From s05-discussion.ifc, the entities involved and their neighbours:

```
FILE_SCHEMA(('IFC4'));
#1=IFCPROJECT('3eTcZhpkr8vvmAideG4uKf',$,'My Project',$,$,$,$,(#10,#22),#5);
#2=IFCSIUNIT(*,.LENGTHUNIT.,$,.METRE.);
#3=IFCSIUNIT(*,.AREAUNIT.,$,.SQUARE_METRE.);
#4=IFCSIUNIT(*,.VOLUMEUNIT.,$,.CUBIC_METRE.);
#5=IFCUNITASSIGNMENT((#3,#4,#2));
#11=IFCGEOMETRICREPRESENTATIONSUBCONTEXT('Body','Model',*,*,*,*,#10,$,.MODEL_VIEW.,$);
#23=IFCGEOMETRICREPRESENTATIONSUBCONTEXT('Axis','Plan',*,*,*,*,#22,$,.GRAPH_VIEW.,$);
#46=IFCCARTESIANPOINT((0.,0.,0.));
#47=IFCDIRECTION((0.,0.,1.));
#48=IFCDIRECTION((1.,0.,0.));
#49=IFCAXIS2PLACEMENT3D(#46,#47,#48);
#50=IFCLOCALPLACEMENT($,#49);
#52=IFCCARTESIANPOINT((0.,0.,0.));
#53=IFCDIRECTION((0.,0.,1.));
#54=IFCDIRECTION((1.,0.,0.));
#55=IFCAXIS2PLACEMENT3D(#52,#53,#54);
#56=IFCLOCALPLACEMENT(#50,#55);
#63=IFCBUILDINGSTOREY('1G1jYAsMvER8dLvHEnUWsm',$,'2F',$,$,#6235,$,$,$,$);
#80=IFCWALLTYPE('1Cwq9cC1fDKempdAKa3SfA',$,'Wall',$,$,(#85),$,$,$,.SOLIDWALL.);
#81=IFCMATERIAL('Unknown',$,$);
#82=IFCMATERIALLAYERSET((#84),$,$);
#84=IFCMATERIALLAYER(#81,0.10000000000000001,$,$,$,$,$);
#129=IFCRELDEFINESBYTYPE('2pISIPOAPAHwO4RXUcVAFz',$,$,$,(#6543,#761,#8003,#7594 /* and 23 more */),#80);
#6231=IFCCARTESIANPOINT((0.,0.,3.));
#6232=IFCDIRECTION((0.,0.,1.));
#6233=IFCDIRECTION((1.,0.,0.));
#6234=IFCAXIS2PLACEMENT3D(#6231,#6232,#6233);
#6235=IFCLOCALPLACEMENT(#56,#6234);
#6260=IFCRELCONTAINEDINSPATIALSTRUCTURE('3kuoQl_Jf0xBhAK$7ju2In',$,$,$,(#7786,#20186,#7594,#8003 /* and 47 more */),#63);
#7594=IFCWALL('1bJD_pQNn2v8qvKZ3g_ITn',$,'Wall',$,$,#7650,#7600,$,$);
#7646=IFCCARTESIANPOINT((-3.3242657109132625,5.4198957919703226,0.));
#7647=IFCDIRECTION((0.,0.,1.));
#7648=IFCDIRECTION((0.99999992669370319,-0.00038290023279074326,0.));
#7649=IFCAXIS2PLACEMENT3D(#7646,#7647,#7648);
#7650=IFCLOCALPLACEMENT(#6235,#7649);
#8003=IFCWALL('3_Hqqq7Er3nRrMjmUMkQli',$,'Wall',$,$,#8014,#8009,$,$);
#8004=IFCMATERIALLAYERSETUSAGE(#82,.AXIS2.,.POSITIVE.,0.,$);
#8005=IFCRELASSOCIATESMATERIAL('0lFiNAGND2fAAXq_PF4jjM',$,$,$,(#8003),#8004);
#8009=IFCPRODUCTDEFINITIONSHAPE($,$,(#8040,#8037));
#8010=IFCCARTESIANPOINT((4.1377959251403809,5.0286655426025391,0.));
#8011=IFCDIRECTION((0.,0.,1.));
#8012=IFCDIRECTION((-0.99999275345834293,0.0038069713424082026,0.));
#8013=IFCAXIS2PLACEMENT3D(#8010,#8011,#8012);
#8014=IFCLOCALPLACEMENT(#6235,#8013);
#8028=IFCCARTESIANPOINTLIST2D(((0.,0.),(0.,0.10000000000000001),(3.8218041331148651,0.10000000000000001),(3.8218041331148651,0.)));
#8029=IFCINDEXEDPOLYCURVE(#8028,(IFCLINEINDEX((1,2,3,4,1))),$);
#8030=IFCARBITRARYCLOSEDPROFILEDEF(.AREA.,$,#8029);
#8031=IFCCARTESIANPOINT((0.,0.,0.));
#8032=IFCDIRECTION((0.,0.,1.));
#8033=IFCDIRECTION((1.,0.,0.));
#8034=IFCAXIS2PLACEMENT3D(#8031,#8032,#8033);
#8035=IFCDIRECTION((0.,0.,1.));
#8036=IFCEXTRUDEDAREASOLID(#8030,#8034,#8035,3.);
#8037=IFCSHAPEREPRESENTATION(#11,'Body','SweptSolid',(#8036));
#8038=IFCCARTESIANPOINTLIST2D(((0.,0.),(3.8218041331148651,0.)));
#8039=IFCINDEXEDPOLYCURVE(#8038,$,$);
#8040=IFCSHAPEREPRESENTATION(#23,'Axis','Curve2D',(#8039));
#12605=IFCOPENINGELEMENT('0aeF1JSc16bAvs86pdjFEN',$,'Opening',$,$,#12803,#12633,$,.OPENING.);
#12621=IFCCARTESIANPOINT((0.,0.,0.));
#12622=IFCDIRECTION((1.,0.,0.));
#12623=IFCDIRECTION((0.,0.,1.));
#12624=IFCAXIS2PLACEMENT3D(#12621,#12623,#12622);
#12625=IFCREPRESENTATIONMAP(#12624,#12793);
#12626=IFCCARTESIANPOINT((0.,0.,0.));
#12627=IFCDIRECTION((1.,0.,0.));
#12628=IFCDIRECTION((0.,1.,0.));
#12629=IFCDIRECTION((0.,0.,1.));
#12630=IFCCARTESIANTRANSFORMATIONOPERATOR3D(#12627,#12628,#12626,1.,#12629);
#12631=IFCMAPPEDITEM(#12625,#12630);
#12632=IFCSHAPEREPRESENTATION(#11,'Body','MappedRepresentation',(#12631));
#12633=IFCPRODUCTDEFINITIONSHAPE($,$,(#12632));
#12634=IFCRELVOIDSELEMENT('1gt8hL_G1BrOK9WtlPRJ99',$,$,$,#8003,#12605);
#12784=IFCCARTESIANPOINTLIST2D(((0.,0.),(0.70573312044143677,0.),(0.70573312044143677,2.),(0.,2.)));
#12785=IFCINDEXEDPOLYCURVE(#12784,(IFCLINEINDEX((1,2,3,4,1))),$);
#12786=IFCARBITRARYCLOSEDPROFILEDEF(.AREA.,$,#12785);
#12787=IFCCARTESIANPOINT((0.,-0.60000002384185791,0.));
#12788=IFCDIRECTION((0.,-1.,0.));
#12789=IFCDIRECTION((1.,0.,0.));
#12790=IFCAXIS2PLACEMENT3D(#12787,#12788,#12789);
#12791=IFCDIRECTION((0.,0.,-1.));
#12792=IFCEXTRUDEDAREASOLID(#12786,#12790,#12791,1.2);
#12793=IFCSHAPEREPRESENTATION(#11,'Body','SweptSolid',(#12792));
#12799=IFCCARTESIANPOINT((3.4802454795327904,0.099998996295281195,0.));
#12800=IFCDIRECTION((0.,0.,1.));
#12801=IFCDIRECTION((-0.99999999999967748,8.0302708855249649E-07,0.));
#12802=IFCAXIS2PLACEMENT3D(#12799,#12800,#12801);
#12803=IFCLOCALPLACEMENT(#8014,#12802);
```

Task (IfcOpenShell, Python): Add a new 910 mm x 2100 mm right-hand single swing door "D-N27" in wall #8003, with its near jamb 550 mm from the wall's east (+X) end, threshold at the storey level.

```python
import numpy as np
import ifcopenshell
import ifcopenshell.api.feature
import ifcopenshell.api.geometry
import ifcopenshell.api.root
import ifcopenshell.api.spatial
import ifcopenshell.geom
import ifcopenshell.util.element
import ifcopenshell.util.placement
import ifcopenshell.util.representation
import ifcopenshell.util.shape
import ifcopenshell.util.unit

model = ifcopenshell.open("s05-discussion.ifc")
unit_scale = ifcopenshell.util.unit.calculate_unit_scale(model)
settings = ifcopenshell.geom.settings()


def volume(element):
    """Net volume in cubic metres, openings subtracted."""
    shape = ifcopenshell.geom.create_shape(settings, element)
    return ifcopenshell.util.shape.get_volume(shape.geometry)


wall = model.by_id(8003)
storey = ifcopenshell.util.element.get_container(wall, ifc_class="IfcBuildingStorey")
context = ifcopenshell.util.representation.get_context(model, "Model", "Body", "MODEL_VIEW")
before = volume(wall)

width, height, from_end, sill = 0.91, 2.1, 0.55, 0.0  # metres

# The wall runs along its own X axis, and the end named is its -X end.
wall_shape = ifcopenshell.geom.create_shape(settings, wall)
x, y, z = ifcopenshell.util.shape.get_vertices(wall_shape.geometry).T
start = x.min() + from_end
face, thickness = float(y.min()), float(y.max() - y.min())
wall_matrix = ifcopenshell.util.placement.get_local_placement(wall.ObjectPlacement)
level = ifcopenshell.util.placement.get_local_placement(storey.ObjectPlacement)[2, 3]


def in_wall(x, y):
    """Placement at x, y metres in the wall's axes, at sill height."""
    matrix = wall_matrix.copy()
    matrix[:, 3] = wall_matrix @ np.array([x / unit_scale, y / unit_scale, 0.0, 1.0])
    matrix[2, 3] = level + sill / unit_scale
    return matrix


# Opening: a box that overshoots both wall faces by 50 mm.
opening = ifcopenshell.api.root.create_entity(model, ifc_class="IfcOpeningElement", predefined_type="OPENING")
box = ifcopenshell.api.geometry.add_wall_representation(
    model, context=context, length=width, height=height, thickness=thickness + 0.1
)
ifcopenshell.api.geometry.assign_representation(model, product=opening, representation=box)
ifcopenshell.api.geometry.edit_object_placement(model, product=opening, matrix=in_wall(start, face - 0.05), is_si=False)
ifcopenshell.api.feature.add_feature(model, feature=opening, element=wall)

door = ifcopenshell.api.root.create_entity(model, ifc_class="IfcDoor", name="D-N27", predefined_type="DOOR")
door.OverallWidth, door.OverallHeight = width / unit_scale, height / unit_scale
door.OperationType = "SINGLE_SWING_RIGHT"
body = ifcopenshell.api.geometry.add_door_representation(
    model,
    context=context,
    overall_width=door.OverallWidth,
    overall_height=door.OverallHeight,
    operation_type="SINGLE_SWING_RIGHT",
    lining_properties={"LiningDepth": thickness / unit_scale, "ThresholdDepth": thickness / unit_scale},
)
ifcopenshell.api.geometry.assign_representation(model, product=door, representation=body)
ifcopenshell.api.spatial.assign_container(model, products=[door], relating_structure=storey)
ifcopenshell.api.feature.add_filling(model, opening=opening, element=door)

# The lining spans the wall, so the door starts at the wall face.
ifcopenshell.api.geometry.edit_object_placement(model, product=door, matrix=in_wall(start, face), is_si=False)

after = volume(wall)

print(f"wall volume {before:.3f} -> {after:.3f} m3")

model.write("s05-discussion-out.ifc")
```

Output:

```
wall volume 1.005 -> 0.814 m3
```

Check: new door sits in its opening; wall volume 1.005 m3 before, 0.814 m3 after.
